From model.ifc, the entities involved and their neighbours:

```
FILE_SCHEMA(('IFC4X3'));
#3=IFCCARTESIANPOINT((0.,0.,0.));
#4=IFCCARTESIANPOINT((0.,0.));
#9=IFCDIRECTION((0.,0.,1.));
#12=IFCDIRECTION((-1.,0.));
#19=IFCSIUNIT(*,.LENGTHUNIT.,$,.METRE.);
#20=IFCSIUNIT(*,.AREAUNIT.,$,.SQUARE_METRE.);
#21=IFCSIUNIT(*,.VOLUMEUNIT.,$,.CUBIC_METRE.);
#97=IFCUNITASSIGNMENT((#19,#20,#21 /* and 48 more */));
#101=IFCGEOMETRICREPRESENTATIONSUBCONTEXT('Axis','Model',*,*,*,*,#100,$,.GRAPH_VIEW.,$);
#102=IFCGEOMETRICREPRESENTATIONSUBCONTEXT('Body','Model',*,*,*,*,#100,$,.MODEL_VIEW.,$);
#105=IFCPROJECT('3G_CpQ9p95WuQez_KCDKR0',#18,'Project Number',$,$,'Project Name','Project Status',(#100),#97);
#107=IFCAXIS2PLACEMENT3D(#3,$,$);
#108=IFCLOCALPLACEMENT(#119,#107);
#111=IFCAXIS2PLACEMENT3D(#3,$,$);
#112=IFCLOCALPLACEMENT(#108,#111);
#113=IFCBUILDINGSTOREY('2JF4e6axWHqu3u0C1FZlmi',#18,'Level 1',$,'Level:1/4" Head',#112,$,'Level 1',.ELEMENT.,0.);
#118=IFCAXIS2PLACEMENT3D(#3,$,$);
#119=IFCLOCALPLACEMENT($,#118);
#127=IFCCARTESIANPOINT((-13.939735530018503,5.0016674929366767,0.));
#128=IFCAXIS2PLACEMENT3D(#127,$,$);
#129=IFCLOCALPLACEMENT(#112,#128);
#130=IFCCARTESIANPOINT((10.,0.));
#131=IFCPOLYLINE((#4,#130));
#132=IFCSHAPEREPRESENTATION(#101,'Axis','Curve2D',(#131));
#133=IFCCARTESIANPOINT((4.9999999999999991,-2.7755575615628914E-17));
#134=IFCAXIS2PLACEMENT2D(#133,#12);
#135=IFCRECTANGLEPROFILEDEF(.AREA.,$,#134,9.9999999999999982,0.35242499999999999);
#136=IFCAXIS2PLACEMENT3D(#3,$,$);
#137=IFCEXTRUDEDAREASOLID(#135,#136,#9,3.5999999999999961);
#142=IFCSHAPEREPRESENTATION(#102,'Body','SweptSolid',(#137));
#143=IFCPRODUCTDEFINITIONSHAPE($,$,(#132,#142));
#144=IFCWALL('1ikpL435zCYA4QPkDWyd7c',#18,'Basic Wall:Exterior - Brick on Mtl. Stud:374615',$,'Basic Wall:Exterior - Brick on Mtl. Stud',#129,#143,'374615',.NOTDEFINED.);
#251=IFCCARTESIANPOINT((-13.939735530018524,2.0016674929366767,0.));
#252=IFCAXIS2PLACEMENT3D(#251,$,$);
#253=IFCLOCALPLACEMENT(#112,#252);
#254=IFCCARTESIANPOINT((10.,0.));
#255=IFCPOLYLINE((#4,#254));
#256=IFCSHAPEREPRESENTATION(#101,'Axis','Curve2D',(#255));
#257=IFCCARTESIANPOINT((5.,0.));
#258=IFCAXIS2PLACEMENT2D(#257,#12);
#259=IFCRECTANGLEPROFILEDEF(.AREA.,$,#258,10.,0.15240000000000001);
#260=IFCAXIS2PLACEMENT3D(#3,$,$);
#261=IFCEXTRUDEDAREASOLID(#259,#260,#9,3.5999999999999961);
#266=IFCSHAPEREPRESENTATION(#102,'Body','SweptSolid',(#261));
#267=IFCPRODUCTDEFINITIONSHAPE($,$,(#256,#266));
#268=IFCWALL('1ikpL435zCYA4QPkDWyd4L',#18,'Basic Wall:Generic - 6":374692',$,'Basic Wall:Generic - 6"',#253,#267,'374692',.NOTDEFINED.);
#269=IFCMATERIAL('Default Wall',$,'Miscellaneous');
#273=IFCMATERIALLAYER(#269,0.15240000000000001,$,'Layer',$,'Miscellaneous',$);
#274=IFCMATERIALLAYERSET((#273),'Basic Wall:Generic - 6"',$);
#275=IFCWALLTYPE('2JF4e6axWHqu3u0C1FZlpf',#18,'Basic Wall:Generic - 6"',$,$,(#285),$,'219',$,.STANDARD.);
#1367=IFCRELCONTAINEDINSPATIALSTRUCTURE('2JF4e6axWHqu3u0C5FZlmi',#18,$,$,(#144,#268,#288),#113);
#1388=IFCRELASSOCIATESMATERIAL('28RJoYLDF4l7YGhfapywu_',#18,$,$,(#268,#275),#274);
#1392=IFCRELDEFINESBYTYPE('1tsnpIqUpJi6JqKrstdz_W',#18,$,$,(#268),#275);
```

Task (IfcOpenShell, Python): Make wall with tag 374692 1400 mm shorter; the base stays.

```python
import ifcopenshell
import ifcopenshell.geom
import ifcopenshell.util.representation
import ifcopenshell.util.shape

model = ifcopenshell.open("model.ifc")
settings = ifcopenshell.geom.settings()


def volume(element):
    """Net volume in cubic metres, openings subtracted."""
    shape = ifcopenshell.geom.create_shape(settings, element)
    return ifcopenshell.util.shape.get_volume(shape.geometry)


wall = model.by_guid("1ikpL435zCYA4QPkDWyd4L")
before = volume(wall)

body = ifcopenshell.util.representation.get_representation(wall, "Model", "Body")
solid = body.Items[0]
old_height = solid.Depth
solid.Depth -= 1.4
after = volume(wall)

print(f"height {old_height:g} -> {solid.Depth:g}, volume {before:.3f} -> {after:.3f} m3")

model.write("model_v2.ifc")
```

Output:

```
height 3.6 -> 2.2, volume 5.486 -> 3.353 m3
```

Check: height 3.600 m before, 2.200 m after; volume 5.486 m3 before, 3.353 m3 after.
